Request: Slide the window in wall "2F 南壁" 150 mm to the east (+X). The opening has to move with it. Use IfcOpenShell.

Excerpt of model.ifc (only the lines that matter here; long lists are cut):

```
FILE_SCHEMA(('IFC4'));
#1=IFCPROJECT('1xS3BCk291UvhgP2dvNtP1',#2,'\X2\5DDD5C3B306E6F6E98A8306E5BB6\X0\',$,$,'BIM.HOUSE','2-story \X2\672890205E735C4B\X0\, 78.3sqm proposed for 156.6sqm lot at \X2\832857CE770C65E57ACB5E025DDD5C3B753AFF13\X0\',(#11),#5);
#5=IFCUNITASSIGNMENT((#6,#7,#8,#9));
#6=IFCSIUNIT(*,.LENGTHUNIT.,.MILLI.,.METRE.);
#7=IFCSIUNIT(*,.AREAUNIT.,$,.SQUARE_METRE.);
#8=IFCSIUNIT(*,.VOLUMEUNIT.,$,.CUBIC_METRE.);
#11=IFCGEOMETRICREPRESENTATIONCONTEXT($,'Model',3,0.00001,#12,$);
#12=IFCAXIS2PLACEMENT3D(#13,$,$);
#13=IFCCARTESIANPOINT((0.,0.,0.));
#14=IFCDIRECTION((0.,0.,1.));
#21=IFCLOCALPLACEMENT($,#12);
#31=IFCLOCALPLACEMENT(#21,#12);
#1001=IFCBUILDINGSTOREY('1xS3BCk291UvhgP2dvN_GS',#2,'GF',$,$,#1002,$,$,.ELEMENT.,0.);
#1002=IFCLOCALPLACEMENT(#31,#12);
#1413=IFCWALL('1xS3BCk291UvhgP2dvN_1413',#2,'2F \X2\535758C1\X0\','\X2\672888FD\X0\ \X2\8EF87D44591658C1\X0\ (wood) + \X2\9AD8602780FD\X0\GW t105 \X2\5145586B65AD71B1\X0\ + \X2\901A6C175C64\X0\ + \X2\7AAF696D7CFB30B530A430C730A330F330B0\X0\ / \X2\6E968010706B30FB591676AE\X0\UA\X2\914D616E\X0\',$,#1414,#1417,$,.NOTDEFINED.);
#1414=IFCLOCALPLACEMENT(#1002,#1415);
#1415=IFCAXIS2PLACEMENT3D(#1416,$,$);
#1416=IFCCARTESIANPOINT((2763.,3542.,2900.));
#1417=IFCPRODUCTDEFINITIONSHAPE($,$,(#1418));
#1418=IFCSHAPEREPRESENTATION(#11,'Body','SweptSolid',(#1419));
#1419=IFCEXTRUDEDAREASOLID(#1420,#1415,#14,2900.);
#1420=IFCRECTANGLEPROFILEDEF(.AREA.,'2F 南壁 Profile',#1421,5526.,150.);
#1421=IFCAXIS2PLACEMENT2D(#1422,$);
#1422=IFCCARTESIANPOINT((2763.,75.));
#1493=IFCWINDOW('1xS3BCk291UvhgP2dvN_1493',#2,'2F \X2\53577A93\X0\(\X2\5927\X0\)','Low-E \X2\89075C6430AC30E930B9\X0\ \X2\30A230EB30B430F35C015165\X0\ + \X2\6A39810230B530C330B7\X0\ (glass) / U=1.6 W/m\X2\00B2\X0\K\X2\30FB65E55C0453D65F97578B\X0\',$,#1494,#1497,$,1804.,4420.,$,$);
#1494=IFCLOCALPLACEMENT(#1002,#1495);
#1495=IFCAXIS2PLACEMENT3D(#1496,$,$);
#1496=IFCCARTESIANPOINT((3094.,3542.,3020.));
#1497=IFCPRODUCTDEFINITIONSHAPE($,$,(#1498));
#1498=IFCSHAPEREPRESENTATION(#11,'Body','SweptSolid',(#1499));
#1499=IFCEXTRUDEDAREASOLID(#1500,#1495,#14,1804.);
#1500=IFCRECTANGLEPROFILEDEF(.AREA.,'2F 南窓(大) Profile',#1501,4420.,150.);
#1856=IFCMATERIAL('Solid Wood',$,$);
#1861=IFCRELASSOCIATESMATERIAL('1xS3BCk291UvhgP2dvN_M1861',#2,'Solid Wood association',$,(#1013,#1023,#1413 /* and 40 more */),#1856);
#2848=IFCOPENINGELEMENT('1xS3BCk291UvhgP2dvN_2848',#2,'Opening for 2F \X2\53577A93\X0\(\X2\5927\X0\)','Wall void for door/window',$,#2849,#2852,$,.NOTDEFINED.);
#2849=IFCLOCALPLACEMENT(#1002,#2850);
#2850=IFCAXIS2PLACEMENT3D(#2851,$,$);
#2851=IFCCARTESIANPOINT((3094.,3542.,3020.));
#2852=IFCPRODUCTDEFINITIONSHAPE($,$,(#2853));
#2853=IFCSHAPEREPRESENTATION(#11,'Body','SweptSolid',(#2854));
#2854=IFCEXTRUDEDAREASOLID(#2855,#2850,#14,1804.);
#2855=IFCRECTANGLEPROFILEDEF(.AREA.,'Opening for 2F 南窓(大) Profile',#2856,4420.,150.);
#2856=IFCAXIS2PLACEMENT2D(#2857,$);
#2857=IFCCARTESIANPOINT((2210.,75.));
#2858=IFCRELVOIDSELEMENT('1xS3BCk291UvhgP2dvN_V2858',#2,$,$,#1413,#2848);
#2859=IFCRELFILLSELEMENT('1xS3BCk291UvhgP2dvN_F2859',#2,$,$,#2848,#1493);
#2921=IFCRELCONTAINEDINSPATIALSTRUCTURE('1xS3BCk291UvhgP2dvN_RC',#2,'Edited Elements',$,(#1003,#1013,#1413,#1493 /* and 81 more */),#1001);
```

```python
import ifcopenshell
import ifcopenshell.api.geometry
import ifcopenshell.util.placement
import ifcopenshell.util.unit

model = ifcopenshell.open("model.ifc")
unit_scale = ifcopenshell.util.unit.calculate_unit_scale(model)

window = model.by_guid("1xS3BCk291UvhgP2dvN_1493")
opening = window.FillsVoids[0].RelatingOpeningElement
wall = opening.VoidsElements[0].RelatingBuildingElement

wall_matrix = ifcopenshell.util.placement.get_local_placement(wall.ObjectPlacement)
shift = wall_matrix[:3, 0] * 0.15 / unit_scale
before = ifcopenshell.util.placement.get_local_placement(window.ObjectPlacement)[:3, 3].copy()

# The window is not placed relative to its opening, so move both.
for product in (opening, window):
    matrix = ifcopenshell.util.placement.get_local_placement(product.ObjectPlacement)
    matrix[:3, 3] += shift
    ifcopenshell.api.geometry.edit_object_placement(model, product=product, matrix=matrix, is_si=False)

after = ifcopenshell.util.placement.get_local_placement(window.ObjectPlacement)[:3, 3]
print("window moved by", (after - before).round(3) + 0.0)

model.write("model-out.ifc")
```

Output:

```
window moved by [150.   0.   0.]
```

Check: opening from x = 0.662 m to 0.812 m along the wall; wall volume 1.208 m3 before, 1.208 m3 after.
